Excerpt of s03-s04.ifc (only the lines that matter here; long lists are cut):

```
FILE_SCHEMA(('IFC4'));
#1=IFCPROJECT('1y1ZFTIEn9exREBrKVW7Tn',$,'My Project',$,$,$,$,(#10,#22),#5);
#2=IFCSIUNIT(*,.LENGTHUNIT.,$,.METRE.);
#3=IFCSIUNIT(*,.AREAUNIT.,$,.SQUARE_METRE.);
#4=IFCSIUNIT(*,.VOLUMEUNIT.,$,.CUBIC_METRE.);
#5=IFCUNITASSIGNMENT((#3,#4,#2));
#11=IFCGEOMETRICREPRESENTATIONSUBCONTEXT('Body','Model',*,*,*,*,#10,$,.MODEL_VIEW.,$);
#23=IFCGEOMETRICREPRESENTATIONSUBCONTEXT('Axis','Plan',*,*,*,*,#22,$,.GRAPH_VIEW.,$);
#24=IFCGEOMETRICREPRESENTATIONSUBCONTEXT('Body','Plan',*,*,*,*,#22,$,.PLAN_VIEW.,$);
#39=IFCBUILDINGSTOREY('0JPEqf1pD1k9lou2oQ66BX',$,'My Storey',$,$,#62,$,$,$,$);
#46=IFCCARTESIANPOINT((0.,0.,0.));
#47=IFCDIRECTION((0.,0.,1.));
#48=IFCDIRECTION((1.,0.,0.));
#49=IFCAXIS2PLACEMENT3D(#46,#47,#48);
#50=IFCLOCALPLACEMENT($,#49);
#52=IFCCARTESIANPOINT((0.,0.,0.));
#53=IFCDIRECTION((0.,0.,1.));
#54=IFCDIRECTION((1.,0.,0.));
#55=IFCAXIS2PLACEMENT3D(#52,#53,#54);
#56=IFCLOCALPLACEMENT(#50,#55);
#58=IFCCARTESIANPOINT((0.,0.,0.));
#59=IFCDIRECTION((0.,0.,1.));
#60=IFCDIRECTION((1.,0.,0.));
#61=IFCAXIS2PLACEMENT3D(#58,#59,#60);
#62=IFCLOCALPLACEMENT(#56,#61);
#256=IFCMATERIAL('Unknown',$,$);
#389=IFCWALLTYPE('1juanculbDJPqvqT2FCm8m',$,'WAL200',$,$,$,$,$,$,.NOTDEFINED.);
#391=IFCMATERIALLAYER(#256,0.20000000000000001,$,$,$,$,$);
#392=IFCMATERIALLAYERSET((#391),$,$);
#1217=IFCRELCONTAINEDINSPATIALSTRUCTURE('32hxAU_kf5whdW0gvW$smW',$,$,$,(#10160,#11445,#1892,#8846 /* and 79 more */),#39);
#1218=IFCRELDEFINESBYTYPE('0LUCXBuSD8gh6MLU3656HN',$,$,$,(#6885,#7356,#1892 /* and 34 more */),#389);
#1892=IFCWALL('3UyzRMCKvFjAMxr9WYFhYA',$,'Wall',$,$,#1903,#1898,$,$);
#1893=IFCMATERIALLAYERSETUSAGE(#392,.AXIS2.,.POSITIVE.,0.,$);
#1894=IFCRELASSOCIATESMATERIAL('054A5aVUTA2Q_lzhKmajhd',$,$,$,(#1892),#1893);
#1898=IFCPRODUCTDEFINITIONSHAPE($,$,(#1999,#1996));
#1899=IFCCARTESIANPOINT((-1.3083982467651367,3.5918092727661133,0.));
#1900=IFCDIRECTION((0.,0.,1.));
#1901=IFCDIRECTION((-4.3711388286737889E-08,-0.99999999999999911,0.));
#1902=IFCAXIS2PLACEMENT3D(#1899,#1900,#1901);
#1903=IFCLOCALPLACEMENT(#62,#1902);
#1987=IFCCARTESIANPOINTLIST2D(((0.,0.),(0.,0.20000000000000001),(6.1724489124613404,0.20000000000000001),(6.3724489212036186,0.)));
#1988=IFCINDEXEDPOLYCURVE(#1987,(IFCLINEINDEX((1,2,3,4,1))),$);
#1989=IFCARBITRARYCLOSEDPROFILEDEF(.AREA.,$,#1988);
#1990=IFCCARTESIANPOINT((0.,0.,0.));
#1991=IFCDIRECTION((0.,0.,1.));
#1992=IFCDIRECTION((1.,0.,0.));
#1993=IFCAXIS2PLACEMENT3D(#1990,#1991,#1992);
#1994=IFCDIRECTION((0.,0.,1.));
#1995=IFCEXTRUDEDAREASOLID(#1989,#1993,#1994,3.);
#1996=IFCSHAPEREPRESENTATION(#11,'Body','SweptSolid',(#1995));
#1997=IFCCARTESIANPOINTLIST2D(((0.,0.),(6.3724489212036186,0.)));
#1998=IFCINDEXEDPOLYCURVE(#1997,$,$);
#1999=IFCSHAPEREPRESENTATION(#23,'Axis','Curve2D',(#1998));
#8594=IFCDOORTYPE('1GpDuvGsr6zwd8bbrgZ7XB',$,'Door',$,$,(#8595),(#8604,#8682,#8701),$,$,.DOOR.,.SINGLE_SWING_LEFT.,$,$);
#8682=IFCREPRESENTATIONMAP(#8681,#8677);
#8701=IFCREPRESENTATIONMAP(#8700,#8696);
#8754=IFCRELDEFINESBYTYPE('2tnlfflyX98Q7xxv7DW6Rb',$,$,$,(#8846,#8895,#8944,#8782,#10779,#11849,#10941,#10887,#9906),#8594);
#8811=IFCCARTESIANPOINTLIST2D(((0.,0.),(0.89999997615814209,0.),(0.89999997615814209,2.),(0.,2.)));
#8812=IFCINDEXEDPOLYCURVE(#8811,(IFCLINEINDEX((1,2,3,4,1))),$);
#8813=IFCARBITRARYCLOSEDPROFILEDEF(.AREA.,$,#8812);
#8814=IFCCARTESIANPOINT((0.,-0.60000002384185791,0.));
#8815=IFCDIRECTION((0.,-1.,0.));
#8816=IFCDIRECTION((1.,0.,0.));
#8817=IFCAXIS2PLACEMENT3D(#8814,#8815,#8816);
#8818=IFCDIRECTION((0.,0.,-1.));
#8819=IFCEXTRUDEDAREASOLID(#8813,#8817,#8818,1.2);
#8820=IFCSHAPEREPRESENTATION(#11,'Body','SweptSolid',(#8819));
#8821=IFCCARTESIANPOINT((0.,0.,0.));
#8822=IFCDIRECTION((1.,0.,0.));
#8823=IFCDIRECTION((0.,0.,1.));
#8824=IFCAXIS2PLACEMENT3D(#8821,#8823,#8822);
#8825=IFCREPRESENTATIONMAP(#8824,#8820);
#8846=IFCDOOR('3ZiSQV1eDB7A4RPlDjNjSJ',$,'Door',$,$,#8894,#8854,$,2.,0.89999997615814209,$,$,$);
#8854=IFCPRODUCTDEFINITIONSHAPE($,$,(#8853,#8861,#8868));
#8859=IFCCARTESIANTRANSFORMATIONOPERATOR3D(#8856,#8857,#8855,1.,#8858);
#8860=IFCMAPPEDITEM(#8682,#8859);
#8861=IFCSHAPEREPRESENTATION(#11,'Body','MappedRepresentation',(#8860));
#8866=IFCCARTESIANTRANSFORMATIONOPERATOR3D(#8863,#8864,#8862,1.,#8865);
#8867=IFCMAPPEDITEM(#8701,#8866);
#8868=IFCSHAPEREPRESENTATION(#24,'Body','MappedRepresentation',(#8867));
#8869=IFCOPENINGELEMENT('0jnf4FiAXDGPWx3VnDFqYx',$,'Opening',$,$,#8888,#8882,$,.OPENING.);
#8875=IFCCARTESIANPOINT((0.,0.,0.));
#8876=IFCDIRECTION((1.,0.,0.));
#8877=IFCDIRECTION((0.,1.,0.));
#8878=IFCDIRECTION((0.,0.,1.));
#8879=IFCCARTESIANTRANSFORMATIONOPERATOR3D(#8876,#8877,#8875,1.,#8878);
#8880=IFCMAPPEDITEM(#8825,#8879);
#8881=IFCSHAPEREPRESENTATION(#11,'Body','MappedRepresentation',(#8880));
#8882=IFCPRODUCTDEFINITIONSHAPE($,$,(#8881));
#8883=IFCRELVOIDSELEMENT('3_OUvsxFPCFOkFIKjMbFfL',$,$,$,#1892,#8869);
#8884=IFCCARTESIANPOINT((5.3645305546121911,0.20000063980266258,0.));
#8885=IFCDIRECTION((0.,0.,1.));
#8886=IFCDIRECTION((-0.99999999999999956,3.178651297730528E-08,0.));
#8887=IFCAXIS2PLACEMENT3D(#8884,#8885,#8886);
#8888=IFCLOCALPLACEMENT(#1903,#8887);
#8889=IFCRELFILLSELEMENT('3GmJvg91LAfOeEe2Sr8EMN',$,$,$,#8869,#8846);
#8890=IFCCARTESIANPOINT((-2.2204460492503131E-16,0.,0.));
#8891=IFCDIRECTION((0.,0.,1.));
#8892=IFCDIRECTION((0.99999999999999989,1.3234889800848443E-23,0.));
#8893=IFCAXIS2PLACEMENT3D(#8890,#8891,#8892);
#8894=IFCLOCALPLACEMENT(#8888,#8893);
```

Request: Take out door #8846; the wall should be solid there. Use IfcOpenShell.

```python
import ifcopenshell
import ifcopenshell.api.feature
import ifcopenshell.api.root
import ifcopenshell.geom
import ifcopenshell.util.shape

model = ifcopenshell.open("s03-s04.ifc")
settings = ifcopenshell.geom.settings()


def volume(element):
    """Net volume in cubic metres, openings subtracted."""
    shape = ifcopenshell.geom.create_shape(settings, element)
    return ifcopenshell.util.shape.get_volume(shape.geometry)


door = model.by_id(8846)
opening = door.FillsVoids[0].RelatingOpeningElement
wall = opening.VoidsElements[0].RelatingBuildingElement
before = volume(wall)

ifcopenshell.api.root.remove_product(model, product=door)
ifcopenshell.api.feature.remove_feature(model, feature=opening)

after = volume(wall)

print(f"wall volume {before:.3f} -> {after:.3f} m3")

model.write("s03-s04-out.ifc")
```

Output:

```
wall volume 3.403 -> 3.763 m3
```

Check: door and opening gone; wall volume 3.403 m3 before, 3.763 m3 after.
